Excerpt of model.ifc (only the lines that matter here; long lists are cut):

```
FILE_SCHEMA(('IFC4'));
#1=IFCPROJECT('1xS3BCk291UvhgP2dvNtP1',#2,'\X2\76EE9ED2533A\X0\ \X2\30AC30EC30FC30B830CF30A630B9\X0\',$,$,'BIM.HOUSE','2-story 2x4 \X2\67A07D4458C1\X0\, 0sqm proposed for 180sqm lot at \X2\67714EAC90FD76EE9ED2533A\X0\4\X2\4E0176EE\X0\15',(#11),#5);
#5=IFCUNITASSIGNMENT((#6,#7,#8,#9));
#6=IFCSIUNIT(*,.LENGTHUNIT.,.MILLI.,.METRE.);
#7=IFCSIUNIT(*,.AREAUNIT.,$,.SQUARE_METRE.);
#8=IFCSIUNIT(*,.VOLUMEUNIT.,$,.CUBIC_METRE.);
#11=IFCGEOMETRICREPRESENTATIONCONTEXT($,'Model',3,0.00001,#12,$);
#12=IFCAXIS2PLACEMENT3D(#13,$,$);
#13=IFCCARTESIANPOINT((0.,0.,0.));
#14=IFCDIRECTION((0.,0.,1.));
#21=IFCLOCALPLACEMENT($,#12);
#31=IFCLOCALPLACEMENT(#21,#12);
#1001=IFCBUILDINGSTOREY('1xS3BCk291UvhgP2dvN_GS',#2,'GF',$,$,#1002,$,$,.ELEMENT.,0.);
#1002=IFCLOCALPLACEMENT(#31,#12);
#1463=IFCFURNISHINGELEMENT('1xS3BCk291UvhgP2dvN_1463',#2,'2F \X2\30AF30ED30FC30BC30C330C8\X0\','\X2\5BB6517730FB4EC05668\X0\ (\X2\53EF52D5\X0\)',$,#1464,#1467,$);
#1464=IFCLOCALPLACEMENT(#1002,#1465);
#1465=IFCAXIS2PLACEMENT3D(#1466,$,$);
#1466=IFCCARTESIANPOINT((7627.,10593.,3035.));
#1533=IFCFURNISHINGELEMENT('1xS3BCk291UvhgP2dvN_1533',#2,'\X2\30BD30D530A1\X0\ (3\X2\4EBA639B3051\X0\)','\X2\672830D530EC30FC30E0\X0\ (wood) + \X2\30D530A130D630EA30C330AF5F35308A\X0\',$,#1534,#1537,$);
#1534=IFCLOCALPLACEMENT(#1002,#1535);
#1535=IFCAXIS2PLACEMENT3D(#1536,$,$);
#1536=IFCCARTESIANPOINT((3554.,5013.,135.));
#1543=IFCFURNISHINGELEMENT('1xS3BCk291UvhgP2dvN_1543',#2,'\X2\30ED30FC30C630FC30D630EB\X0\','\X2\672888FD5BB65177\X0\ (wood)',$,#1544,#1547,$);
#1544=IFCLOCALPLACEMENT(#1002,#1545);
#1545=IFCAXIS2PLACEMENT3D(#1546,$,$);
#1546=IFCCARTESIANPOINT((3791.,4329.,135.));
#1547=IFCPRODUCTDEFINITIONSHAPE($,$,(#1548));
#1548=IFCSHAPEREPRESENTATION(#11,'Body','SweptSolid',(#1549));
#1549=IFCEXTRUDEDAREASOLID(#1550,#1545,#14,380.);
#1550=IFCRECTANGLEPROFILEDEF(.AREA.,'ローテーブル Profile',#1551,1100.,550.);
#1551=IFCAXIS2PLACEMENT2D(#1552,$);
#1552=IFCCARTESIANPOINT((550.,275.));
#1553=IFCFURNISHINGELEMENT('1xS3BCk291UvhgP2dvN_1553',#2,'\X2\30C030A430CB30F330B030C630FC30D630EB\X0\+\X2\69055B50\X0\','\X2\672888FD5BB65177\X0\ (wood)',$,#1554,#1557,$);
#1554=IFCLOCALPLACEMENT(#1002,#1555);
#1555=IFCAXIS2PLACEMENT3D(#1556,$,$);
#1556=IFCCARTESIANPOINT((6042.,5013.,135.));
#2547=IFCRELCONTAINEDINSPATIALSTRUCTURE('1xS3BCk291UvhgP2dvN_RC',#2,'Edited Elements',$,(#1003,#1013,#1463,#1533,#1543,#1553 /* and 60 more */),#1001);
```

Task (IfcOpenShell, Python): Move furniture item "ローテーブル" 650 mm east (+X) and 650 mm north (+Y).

```python
import ifcopenshell
import ifcopenshell.api.geometry
import ifcopenshell.util.placement
import ifcopenshell.util.unit

model = ifcopenshell.open("model.ifc")
unit_scale = ifcopenshell.util.unit.calculate_unit_scale(model)

item = model.by_id(1543)
matrix = ifcopenshell.util.placement.get_local_placement(item.ObjectPlacement)
matrix[0, 3] += 0.65 / unit_scale
matrix[1, 3] += 0.65 / unit_scale
ifcopenshell.api.geometry.edit_object_placement(model, product=item, matrix=matrix, is_si=False)

print(ifcopenshell.util.placement.get_local_placement(item.ObjectPlacement).round(3) + 0.0)

model.write("model_v2.ifc")
```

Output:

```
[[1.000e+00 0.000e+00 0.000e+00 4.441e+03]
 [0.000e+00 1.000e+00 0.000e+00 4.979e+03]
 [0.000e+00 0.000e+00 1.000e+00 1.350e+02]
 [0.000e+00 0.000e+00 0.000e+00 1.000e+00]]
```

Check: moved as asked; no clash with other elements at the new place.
